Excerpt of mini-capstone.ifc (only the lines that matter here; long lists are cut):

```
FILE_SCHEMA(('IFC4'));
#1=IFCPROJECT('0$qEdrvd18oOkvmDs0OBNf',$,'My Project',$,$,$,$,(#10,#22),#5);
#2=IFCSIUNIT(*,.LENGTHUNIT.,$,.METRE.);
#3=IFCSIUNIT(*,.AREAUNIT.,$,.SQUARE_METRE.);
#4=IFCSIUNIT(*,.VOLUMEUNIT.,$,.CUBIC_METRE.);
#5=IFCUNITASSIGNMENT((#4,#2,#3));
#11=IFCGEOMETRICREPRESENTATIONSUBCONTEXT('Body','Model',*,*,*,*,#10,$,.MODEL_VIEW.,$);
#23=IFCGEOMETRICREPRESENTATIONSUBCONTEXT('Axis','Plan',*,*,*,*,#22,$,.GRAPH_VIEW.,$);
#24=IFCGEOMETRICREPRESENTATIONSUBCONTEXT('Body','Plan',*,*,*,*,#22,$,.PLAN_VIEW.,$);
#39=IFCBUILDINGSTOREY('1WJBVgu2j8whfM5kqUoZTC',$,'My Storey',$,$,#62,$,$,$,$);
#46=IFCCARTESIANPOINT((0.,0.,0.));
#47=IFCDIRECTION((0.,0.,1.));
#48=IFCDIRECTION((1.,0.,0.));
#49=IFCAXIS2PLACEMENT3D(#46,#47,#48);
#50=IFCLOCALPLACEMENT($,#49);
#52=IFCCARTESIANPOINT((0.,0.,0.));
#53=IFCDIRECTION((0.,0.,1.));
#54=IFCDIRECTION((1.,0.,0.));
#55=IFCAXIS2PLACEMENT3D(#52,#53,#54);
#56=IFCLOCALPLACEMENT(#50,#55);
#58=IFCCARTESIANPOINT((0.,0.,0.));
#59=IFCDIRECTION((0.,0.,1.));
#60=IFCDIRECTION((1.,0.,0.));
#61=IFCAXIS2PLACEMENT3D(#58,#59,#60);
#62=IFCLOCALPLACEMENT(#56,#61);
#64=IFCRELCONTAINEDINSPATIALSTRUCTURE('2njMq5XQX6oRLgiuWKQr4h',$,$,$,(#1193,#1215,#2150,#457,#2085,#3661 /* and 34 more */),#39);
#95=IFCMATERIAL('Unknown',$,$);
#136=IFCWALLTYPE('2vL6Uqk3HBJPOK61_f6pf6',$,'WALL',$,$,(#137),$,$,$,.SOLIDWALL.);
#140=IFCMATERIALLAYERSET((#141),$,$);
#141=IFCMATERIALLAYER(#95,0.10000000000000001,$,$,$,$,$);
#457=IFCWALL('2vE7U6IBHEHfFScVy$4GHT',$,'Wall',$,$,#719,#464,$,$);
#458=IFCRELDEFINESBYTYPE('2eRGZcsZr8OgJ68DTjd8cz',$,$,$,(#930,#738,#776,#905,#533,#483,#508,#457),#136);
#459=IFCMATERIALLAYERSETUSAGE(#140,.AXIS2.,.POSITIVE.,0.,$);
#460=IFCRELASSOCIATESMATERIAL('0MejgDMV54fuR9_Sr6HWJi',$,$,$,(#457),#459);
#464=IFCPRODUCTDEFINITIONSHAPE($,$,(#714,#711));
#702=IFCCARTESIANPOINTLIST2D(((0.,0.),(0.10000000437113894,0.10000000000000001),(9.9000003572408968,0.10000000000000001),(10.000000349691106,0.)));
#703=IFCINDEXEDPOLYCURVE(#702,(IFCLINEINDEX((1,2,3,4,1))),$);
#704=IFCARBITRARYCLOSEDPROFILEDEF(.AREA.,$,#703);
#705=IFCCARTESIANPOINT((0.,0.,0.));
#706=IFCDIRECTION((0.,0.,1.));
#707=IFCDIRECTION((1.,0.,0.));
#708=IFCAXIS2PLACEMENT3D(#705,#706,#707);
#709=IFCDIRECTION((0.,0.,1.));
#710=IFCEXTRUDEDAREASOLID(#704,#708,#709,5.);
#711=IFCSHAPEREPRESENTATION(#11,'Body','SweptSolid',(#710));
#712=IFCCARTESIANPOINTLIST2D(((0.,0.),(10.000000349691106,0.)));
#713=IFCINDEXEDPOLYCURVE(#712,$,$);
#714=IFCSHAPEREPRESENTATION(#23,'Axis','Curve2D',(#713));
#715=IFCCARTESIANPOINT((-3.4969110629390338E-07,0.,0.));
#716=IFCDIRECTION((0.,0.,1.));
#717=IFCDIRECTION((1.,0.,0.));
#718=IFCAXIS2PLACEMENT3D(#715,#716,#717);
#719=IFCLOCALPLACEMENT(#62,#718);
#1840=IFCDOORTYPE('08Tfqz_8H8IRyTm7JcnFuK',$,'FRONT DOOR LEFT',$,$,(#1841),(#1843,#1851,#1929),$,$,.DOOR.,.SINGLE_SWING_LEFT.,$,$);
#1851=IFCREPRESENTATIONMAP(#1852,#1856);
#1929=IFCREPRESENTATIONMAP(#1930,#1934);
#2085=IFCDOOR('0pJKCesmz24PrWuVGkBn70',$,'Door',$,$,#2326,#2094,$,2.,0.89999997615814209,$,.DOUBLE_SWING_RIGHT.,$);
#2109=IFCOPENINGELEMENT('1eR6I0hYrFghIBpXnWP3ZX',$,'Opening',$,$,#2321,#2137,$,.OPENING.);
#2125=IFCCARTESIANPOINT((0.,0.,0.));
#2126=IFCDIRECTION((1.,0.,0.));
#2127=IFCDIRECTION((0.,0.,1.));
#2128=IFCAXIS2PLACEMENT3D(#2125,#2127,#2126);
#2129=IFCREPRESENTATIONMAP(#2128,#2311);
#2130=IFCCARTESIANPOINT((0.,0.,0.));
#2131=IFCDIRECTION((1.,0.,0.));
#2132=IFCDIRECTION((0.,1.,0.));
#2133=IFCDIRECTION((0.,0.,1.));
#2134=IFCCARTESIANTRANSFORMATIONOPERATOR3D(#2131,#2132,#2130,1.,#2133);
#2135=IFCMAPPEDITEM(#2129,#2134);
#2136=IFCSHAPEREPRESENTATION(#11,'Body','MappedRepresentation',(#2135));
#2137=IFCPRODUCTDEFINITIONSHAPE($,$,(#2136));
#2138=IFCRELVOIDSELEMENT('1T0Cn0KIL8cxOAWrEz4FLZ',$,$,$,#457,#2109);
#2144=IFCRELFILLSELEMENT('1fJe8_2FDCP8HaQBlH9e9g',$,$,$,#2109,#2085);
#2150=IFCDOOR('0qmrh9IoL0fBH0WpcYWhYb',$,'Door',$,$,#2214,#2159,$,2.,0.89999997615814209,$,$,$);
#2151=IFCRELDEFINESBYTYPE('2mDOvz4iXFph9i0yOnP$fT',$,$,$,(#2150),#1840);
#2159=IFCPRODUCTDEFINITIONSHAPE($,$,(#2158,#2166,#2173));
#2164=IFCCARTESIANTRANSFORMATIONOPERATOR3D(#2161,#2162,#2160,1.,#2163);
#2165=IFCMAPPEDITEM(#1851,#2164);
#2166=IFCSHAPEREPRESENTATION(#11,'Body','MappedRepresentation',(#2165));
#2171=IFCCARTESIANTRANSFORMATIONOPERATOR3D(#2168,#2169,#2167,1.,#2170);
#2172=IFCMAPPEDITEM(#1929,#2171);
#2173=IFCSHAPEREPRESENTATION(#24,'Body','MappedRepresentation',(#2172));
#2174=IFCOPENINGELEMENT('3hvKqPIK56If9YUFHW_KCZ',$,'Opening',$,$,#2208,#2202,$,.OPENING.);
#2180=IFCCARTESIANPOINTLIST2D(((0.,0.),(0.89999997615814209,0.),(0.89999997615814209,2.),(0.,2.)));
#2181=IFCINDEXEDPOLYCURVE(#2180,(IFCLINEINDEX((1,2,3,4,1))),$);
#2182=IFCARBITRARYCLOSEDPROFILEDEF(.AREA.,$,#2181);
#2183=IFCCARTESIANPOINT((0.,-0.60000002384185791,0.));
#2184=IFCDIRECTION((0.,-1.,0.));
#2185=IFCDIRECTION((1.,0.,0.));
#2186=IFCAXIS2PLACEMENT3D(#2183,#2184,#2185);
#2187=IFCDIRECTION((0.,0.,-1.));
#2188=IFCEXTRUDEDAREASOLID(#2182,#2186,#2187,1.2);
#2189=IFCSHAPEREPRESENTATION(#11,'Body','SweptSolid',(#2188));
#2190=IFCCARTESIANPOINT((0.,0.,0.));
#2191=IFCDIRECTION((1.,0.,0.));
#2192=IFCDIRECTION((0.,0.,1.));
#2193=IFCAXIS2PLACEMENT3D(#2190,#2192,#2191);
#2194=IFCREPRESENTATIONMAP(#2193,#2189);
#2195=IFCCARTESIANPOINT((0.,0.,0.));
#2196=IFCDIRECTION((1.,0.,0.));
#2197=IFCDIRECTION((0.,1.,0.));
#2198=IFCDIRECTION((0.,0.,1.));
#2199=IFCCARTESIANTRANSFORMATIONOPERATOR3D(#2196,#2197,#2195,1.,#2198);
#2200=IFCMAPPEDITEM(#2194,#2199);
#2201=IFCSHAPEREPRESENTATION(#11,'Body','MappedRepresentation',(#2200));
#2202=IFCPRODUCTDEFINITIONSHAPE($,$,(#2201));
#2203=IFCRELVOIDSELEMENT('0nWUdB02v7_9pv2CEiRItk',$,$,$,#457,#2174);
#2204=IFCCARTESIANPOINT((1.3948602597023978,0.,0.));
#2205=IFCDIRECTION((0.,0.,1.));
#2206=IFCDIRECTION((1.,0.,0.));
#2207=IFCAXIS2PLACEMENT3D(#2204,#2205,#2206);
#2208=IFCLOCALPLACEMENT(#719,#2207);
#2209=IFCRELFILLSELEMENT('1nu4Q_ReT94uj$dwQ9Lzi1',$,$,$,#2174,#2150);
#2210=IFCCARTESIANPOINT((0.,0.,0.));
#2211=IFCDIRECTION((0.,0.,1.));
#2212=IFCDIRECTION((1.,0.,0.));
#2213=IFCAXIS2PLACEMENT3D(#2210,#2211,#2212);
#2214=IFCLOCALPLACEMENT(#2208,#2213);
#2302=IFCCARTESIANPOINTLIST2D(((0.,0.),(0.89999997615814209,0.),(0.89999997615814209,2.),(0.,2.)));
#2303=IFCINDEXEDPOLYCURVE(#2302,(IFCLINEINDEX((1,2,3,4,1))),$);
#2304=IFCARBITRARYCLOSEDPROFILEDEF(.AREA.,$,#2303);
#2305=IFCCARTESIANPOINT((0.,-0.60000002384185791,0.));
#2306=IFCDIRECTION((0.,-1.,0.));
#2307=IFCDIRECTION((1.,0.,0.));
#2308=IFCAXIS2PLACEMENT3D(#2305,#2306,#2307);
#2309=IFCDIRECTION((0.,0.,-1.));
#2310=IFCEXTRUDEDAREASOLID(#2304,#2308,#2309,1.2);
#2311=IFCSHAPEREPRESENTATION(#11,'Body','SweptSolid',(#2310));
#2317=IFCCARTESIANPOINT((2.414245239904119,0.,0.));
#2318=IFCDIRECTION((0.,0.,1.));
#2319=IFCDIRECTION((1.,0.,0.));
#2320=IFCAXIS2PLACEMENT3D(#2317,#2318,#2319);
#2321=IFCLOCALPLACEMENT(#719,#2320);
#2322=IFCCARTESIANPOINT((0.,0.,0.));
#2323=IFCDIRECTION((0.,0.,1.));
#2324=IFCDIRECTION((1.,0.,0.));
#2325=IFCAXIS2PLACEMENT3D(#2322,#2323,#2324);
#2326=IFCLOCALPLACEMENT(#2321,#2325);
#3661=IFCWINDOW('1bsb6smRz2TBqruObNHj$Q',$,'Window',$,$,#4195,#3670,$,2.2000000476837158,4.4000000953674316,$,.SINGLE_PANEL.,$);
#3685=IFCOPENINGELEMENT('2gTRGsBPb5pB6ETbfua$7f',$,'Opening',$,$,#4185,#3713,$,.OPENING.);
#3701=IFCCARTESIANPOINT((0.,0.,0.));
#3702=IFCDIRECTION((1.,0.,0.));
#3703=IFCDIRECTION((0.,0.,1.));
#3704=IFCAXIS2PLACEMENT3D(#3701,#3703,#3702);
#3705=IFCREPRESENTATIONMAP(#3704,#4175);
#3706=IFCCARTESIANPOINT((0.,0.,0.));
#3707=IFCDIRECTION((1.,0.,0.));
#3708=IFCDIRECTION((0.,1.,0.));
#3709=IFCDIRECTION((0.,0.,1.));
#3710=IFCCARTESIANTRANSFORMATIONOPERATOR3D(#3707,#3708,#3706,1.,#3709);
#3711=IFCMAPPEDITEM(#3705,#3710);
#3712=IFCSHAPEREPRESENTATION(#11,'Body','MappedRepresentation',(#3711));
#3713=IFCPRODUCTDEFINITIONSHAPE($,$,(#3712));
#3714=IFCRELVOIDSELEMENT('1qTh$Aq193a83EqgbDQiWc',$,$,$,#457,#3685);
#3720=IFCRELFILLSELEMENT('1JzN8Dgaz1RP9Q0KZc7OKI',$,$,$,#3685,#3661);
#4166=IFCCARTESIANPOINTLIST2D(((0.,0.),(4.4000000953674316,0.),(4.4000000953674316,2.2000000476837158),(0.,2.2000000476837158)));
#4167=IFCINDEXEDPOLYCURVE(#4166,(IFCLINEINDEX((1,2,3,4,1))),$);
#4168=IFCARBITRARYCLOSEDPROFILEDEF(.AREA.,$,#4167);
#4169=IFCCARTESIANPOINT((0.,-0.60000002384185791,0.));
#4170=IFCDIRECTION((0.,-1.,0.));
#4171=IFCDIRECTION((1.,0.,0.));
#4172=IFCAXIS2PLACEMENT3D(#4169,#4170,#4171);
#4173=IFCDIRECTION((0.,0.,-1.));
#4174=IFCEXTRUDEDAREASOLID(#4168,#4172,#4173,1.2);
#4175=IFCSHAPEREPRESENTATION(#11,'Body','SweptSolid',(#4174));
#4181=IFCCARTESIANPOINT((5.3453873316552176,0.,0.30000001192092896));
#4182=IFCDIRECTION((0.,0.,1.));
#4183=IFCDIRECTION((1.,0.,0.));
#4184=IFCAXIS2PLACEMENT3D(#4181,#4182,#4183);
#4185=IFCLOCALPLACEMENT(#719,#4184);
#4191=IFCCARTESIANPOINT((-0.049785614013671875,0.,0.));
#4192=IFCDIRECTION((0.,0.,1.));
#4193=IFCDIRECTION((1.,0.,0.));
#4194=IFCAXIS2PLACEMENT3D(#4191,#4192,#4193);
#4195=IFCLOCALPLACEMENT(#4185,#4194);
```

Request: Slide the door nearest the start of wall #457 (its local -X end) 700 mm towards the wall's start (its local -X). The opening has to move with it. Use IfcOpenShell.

```python
import ifcopenshell
import ifcopenshell.api.geometry
import ifcopenshell.util.placement
import ifcopenshell.util.unit

model = ifcopenshell.open("mini-capstone.ifc")
unit_scale = ifcopenshell.util.unit.calculate_unit_scale(model)

door = model.by_id(2150)
opening = door.FillsVoids[0].RelatingOpeningElement
wall = opening.VoidsElements[0].RelatingBuildingElement

wall_matrix = ifcopenshell.util.placement.get_local_placement(wall.ObjectPlacement)
shift = wall_matrix[:3, 0] * -0.7 / unit_scale
before = ifcopenshell.util.placement.get_local_placement(door.ObjectPlacement)[:3, 3].copy()

# The door is placed relative to its opening, so it follows when the opening moves.
matrix = ifcopenshell.util.placement.get_local_placement(opening.ObjectPlacement)
matrix[:3, 3] += shift
ifcopenshell.api.geometry.edit_object_placement(
    model, product=opening, matrix=matrix, is_si=False, should_transform_children=True
)

after = ifcopenshell.util.placement.get_local_placement(door.ObjectPlacement)[:3, 3]
print("door moved by", (after - before).round(3) + 0.0)

model.write("mini-capstone-out.ifc")
```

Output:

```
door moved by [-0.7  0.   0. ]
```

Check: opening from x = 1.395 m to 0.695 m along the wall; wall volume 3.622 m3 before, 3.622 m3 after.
